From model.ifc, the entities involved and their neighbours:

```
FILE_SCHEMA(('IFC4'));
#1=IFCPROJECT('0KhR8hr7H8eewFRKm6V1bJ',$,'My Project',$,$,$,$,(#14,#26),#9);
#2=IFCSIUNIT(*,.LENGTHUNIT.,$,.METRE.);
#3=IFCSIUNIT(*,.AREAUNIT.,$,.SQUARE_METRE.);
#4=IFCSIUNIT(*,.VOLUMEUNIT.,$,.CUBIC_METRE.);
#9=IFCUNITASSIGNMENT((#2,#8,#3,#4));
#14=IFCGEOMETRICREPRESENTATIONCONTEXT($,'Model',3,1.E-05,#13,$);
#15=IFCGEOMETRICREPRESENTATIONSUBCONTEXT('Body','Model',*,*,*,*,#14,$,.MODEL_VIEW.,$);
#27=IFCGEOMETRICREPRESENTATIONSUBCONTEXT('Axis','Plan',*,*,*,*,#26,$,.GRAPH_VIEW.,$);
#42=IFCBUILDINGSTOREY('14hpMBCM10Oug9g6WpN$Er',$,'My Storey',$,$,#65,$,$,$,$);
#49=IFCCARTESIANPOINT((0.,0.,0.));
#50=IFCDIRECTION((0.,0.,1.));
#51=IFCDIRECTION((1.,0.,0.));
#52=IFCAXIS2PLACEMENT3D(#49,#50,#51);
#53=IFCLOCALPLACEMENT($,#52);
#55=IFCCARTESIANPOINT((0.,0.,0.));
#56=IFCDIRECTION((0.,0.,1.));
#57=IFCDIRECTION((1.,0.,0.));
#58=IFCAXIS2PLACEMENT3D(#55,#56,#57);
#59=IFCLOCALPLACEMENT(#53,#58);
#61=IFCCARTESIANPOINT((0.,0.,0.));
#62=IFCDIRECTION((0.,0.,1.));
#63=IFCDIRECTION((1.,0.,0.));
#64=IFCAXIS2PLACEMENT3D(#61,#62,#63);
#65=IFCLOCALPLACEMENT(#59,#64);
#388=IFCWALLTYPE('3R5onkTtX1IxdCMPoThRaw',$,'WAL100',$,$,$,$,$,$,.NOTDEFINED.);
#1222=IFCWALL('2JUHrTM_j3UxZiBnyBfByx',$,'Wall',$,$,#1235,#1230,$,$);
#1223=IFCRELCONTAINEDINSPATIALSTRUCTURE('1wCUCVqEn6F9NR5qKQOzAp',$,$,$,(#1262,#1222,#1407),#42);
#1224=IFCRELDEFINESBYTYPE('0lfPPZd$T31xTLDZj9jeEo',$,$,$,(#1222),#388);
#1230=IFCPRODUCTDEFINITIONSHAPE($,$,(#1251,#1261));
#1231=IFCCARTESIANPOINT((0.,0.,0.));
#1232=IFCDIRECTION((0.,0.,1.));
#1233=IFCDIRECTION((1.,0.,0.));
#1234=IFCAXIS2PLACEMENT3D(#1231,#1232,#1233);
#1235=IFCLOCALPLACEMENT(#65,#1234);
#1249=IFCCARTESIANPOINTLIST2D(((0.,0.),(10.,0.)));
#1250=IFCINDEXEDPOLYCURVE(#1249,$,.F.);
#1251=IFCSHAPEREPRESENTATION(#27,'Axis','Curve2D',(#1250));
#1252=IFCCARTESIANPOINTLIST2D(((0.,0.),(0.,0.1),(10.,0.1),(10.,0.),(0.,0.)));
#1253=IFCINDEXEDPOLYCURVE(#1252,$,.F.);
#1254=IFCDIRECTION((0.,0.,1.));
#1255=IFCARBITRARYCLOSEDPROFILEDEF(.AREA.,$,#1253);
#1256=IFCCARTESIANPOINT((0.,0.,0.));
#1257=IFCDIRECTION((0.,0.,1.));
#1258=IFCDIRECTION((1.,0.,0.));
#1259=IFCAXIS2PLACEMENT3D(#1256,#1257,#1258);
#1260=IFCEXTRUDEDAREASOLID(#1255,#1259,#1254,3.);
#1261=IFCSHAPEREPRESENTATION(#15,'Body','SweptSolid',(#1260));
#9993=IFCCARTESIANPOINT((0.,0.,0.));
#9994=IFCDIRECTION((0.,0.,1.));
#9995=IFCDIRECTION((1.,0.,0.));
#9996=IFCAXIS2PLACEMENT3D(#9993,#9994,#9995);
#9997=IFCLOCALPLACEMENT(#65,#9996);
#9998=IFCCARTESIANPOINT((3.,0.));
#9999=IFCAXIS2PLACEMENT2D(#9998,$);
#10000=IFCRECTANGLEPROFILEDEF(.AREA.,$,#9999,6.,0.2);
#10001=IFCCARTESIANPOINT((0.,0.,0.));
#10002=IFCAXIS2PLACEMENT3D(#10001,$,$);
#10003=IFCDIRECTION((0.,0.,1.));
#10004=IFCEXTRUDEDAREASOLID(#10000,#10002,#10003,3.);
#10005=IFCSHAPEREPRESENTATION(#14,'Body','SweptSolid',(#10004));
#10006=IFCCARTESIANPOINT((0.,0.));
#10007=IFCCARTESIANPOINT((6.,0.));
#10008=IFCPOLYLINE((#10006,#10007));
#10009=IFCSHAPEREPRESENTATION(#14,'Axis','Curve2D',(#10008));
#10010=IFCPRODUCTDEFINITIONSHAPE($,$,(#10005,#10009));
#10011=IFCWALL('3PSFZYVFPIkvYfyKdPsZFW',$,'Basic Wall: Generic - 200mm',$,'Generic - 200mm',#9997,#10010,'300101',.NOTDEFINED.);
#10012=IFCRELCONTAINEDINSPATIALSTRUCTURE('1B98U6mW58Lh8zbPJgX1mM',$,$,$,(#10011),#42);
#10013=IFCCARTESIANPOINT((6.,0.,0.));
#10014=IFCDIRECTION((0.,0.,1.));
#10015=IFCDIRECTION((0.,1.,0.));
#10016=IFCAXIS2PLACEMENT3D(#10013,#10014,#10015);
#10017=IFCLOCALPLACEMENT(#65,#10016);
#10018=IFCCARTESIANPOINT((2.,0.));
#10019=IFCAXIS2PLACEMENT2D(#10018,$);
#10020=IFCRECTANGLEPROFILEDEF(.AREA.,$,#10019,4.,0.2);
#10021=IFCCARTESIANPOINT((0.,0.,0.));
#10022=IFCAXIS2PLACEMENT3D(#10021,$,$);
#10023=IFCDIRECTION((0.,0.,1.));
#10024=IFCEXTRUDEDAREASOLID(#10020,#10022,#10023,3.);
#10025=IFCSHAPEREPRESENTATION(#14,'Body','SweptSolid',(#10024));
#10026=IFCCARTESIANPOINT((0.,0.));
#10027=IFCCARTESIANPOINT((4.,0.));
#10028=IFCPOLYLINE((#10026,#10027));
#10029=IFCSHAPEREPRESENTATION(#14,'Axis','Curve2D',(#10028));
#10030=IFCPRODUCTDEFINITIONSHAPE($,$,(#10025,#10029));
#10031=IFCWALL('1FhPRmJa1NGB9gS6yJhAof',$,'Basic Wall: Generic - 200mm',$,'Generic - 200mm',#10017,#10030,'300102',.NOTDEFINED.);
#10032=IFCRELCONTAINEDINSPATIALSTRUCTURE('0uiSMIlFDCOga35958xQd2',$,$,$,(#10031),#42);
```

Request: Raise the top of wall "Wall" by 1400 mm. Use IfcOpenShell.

```python
import ifcopenshell
import ifcopenshell.geom
import ifcopenshell.util.representation
import ifcopenshell.util.shape
import ifcopenshell.util.unit

model = ifcopenshell.open("model.ifc")
unit_scale = ifcopenshell.util.unit.calculate_unit_scale(model)
settings = ifcopenshell.geom.settings()


def volume(element):
    """Net volume in cubic metres, openings subtracted."""
    shape = ifcopenshell.geom.create_shape(settings, element)
    return ifcopenshell.util.shape.get_volume(shape.geometry)


wall = model.by_guid("2JUHrTM_j3UxZiBnyBfByx")
before = volume(wall)

body = ifcopenshell.util.representation.get_representation(wall, "Model", "Body")
solid = body.Items[0]
old_height = solid.Depth
solid.Depth += 1.4 / unit_scale
after = volume(wall)

print(f"height {old_height:g} -> {solid.Depth:g}, volume {before:.3f} -> {after:.3f} m3")

model.write("model_rev.ifc")
```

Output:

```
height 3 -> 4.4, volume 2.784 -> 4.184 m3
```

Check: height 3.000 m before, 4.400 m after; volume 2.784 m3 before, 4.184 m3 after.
